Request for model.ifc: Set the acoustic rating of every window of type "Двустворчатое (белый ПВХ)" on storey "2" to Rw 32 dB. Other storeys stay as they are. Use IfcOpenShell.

First a look at what the model holds.

```python
import ifcopenshell
import ifcopenshell.util.element

model = ifcopenshell.open("model.ifc")
print(model.schema)
storey = next(s for s in model.by_type("IfcBuildingStorey") if s.Name == "2")
windows = [e for e in ifcopenshell.util.element.get_decomposition(storey) if e.is_a("IfcWindow")]
seen = {}
for e in windows:
    element_type = ifcopenshell.util.element.get_type(e)
    key = (element_type.Name if element_type != e and element_type else None, ifcopenshell.util.element.get_pset(e, "Pset_WindowCommon", "AcousticRating"))
    seen[key] = seen.get(key, 0) + 1
for (name, value), count in sorted(seen.items(), key=str):
    print(count, "x", name, "|", value)
```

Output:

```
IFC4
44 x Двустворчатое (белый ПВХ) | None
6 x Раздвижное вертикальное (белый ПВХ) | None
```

```python
import ifcopenshell
import ifcopenshell.api.pset
import ifcopenshell.util.element

model = ifcopenshell.open("model.ifc")

storey = next(s for s in model.by_type("IfcBuildingStorey") if s.Name == "2")
windows = [e for e in ifcopenshell.util.element.get_decomposition(storey) if e.is_a("IfcWindow")]

count = 0
for e in windows:
    element_type = ifcopenshell.util.element.get_type(e)
    if element_type in (None, e) or element_type.Name != "Двустворчатое (белый ПВХ)":
        continue
    # add_pset returns the element's existing set when there is one.
    pset = ifcopenshell.api.pset.add_pset(model, product=e, name="Pset_WindowCommon")
    ifcopenshell.api.pset.edit_pset(model, pset=pset, properties={"AcousticRating": "Rw 32 dB"})
    count += 1

print(count, "windows updated")

model.write("model_rev.ifc")
```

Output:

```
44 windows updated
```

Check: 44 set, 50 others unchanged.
